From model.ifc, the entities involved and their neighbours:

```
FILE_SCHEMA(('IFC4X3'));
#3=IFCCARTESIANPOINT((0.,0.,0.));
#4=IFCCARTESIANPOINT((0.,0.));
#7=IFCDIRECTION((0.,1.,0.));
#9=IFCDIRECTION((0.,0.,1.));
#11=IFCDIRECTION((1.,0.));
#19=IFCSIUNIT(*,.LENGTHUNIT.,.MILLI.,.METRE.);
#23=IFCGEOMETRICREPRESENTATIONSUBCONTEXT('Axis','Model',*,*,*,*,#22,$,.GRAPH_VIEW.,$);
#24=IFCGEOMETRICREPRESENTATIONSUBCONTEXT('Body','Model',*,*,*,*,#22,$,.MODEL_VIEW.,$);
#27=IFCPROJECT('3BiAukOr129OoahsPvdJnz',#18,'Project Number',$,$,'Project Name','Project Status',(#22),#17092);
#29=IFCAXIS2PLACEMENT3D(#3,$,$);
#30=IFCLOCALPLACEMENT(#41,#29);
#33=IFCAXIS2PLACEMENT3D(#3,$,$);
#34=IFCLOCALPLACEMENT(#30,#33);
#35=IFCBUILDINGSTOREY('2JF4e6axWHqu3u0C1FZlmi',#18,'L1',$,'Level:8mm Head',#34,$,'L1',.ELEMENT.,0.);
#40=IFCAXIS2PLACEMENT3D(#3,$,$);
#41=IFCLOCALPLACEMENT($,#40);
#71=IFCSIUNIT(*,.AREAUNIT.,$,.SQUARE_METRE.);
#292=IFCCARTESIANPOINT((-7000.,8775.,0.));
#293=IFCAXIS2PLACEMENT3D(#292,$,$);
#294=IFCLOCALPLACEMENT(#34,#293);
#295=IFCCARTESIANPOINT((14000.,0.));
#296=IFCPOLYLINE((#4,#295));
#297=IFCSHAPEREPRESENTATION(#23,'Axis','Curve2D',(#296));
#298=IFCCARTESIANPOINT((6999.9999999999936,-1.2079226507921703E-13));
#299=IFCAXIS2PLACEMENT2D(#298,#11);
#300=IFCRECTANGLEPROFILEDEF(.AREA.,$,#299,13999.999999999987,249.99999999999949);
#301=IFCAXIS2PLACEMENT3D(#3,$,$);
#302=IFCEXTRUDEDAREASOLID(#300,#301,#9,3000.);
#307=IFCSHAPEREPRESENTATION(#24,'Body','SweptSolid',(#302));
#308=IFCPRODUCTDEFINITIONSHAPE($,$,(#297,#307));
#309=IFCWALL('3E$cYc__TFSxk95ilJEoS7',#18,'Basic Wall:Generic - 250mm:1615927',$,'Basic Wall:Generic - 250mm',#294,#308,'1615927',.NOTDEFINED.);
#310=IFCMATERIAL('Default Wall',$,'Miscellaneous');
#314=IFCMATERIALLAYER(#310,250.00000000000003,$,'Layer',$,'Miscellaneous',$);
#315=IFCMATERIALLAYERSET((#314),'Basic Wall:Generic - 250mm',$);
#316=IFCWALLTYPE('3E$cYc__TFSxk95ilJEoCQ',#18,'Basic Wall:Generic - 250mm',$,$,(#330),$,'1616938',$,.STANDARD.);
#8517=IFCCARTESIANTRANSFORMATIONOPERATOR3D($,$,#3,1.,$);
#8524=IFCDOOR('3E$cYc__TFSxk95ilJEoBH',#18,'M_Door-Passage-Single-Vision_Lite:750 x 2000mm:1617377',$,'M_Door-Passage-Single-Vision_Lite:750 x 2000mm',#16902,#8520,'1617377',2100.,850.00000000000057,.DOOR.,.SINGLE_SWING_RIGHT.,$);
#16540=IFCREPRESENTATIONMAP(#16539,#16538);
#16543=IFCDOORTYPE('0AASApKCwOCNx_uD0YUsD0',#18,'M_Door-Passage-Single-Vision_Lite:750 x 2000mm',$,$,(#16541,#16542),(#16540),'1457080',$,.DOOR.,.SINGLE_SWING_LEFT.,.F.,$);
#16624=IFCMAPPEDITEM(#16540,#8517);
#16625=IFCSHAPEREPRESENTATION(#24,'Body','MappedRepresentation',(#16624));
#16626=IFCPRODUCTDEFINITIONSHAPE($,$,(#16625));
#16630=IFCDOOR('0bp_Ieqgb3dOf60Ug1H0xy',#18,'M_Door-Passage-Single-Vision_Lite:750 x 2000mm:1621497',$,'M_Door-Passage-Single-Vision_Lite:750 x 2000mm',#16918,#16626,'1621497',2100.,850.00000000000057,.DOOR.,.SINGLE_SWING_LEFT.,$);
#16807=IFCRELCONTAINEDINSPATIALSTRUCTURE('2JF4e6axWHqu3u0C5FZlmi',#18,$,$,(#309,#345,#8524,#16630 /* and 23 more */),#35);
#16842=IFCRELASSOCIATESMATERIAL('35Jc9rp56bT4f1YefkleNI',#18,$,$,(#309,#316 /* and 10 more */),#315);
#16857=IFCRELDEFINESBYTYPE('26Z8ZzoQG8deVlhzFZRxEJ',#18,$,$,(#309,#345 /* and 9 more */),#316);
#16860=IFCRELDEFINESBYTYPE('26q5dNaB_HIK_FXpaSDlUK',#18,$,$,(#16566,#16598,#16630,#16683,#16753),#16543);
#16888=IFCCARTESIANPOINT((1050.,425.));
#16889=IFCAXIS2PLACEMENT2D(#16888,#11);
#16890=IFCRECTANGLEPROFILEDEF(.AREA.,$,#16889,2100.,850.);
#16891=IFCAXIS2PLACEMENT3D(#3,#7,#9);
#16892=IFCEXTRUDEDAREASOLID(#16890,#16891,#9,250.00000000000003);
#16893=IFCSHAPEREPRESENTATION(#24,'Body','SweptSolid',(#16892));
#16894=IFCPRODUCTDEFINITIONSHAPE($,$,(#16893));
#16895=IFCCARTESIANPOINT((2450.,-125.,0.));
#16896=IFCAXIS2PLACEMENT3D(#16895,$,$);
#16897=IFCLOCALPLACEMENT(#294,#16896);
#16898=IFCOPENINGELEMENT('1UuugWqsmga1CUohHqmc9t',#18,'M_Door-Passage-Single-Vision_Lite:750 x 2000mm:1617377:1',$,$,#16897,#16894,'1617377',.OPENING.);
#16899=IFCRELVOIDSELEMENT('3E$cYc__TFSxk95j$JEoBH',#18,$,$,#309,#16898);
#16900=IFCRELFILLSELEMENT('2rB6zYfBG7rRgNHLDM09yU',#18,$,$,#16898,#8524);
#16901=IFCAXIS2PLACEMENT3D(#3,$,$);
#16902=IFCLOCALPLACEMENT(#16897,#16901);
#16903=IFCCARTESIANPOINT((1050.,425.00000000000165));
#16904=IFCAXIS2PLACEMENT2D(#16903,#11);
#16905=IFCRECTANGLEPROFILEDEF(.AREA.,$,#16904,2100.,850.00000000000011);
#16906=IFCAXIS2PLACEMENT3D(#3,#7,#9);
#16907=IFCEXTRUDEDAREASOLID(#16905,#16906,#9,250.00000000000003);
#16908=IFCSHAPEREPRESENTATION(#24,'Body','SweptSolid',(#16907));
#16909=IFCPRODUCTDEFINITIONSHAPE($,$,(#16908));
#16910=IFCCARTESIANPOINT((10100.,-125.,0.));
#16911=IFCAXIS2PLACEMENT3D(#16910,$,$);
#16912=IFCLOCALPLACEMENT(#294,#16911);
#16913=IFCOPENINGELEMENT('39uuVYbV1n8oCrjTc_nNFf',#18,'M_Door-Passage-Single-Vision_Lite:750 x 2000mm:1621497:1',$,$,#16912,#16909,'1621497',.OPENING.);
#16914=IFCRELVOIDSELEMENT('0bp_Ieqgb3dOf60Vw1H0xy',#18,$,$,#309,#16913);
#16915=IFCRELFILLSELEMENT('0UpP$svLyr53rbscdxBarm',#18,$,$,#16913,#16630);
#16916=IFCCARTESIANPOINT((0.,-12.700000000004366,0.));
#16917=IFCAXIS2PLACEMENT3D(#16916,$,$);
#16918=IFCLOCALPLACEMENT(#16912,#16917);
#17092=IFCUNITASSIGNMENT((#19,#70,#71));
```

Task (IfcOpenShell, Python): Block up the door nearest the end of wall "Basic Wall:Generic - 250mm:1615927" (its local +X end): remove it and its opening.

```python
import ifcopenshell
import ifcopenshell.api.feature
import ifcopenshell.api.root
import ifcopenshell.geom
import ifcopenshell.util.shape

model = ifcopenshell.open("model.ifc")
settings = ifcopenshell.geom.settings()


def volume(element):
    """Net volume in cubic metres, openings subtracted."""
    shape = ifcopenshell.geom.create_shape(settings, element)
    return ifcopenshell.util.shape.get_volume(shape.geometry)


door = model.by_guid("0bp_Ieqgb3dOf60Ug1H0xy")
opening = door.FillsVoids[0].RelatingOpeningElement
wall = opening.VoidsElements[0].RelatingBuildingElement
before = volume(wall)

ifcopenshell.api.root.remove_product(model, product=door)
ifcopenshell.api.feature.remove_feature(model, feature=opening)

after = volume(wall)

print(f"wall volume {before:.3f} -> {after:.3f} m3")

model.write("model_rev.ifc")
```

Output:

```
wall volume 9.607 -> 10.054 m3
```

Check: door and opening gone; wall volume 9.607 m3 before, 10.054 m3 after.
